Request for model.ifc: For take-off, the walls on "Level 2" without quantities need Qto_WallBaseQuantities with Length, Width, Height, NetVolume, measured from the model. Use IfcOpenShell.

First a look at what the model holds.

```python
import ifcopenshell
import ifcopenshell.util.element
import ifcopenshell.util.unit

model = ifcopenshell.open("model.ifc")
print(model.schema)
for unit_type in ("LENGTHUNIT", "AREAUNIT", "VOLUMEUNIT"):
    print(unit_type, ifcopenshell.util.unit.calculate_unit_scale(model, unit_type))
storey = next(s for s in model.by_type("IfcBuildingStorey") if s.Name == "Level 2")
walls = [e for e in ifcopenshell.util.element.get_decomposition(storey) if e.is_a("IfcWall")]
for e in sorted(walls, key=lambda e: e.id()):
    print(e.id(), e.is_a(), e.Name, list(ifcopenshell.util.element.get_psets(e, qtos_only=True)), sep=" | ")
```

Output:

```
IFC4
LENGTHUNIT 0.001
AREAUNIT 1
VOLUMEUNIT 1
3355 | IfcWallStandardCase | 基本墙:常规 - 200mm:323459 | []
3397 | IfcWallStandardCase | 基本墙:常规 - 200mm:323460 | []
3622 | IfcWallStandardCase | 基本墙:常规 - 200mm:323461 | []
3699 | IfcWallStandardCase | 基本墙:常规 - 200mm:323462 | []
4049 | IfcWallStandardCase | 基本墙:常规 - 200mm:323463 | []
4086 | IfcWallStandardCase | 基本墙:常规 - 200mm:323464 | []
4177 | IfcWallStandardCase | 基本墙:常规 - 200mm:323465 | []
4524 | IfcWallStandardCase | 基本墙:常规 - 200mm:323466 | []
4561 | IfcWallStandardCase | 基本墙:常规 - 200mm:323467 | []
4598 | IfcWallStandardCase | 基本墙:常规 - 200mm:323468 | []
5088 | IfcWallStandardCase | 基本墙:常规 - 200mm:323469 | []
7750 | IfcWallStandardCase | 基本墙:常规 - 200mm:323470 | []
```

```python
import ifcopenshell
import ifcopenshell.api.pset
import ifcopenshell.geom
import ifcopenshell.util.element
import ifcopenshell.util.shape
import ifcopenshell.util.unit

model = ifcopenshell.open("model.ifc")
unit_scale = ifcopenshell.util.unit.calculate_unit_scale(model)
volume_scale = ifcopenshell.util.unit.calculate_unit_scale(model, "VOLUMEUNIT")
settings = ifcopenshell.geom.settings()

storey = next(s for s in model.by_type("IfcBuildingStorey") if s.Name == "Level 2")
walls = [e for e in ifcopenshell.util.element.get_decomposition(storey) if e.is_a("IfcWall")]

for e in sorted(walls, key=lambda e: e.id()):
    if ifcopenshell.util.element.get_psets(e, qtos_only=True, should_inherit=False):
        continue
    # Geometry comes back in metres, in the element's own axes.
    shape = ifcopenshell.geom.create_shape(settings, e)
    values = {
        "Length": ifcopenshell.util.shape.get_x(shape.geometry) / unit_scale,
        "Width": ifcopenshell.util.shape.get_y(shape.geometry) / unit_scale,
        "Height": ifcopenshell.util.shape.get_z(shape.geometry) / unit_scale,
        "NetVolume": ifcopenshell.util.shape.get_volume(shape.geometry) / volume_scale,
    }
    qto = ifcopenshell.api.pset.add_qto(model, product=e, name="Qto_WallBaseQuantities")
    ifcopenshell.api.pset.edit_qto(model, qto=qto, properties=values)
    print(e.id(), {k: round(v, 3) for k, v in values.items()})

model.write("model-out.ifc")
```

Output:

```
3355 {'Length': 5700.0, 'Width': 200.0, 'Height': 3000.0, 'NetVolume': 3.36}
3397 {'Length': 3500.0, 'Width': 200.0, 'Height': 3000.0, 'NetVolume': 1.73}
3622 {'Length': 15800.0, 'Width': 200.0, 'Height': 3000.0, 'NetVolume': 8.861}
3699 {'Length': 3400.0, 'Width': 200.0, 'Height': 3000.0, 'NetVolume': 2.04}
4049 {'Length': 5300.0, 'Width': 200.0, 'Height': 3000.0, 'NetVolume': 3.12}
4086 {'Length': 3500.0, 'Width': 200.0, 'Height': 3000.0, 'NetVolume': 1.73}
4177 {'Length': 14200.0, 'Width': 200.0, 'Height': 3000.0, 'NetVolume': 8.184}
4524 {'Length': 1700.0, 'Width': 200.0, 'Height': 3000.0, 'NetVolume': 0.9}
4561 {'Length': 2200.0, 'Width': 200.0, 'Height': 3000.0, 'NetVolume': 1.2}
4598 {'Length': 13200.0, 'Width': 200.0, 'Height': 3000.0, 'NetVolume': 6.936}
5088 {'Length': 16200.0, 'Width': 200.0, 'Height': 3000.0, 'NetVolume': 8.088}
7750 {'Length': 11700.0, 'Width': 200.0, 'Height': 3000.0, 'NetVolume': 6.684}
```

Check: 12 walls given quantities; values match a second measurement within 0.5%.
